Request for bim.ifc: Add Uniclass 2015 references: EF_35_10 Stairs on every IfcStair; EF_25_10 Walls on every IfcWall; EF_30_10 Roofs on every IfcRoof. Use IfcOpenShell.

First a look at what the model holds.

```python
import ifcopenshell

model = ifcopenshell.open("bim.ifc")
print(model.schema)
print("classifications:", [c.Name for c in model.by_type("IfcClassification")])
for ifc_class in ("IfcDoor", "IfcRoof", "IfcStair", "IfcWall", "IfcWindow"):
    print(ifc_class, len(model.by_type(ifc_class)))
```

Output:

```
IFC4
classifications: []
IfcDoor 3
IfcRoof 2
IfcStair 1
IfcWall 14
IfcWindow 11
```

```python
import ifcopenshell
import ifcopenshell.api.classification

model = ifcopenshell.open("bim.ifc")

system = ifcopenshell.api.classification.add_classification(model, classification="Uniclass 2015")

codes = {
    "IfcStair": ("EF_35_10", "Stairs"),
    "IfcWall": ("EF_25_10", "Walls"),
    "IfcRoof": ("EF_30_10", "Roofs"),
}
for ifc_class, (code, name) in codes.items():
    products = model.by_type(ifc_class)
    ifcopenshell.api.classification.add_reference(
        model, products=products, classification=system, identification=code, name=name
    )
    print(code, len(products))

model.write("bim-out.ifc")
```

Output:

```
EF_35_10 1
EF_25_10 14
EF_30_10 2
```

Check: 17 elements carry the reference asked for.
